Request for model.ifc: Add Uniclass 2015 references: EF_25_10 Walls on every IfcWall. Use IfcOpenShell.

First a look at what the model holds.

```python
import ifcopenshell

model = ifcopenshell.open("model.ifc")
print(model.schema)
print("classifications:", [c.Name for c in model.by_type("IfcClassification")])
for ifc_class in ("IfcDoor", "IfcRoof", "IfcStair", "IfcWall", "IfcWindow"):
    print(ifc_class, len(model.by_type(ifc_class)))
```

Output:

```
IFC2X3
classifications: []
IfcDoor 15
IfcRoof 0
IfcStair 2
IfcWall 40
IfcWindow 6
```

```python
import ifcopenshell
import ifcopenshell.api.classification

model = ifcopenshell.open("model.ifc")

# IFC2X3 requires Source and Edition and has no link from the project to the system.
system = model.create_entity("IfcClassification", Source="NBS", Edition="2015", Name="Uniclass 2015")

codes = {
    "IfcWall": ("EF_25_10", "Walls"),
}
for ifc_class, (code, name) in codes.items():
    products = model.by_type(ifc_class)
    ifcopenshell.api.classification.add_reference(
        model, products=products, classification=system, identification=code, name=name
    )
    print(code, len(products))

model.write("model-out.ifc")
```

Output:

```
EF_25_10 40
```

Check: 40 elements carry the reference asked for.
